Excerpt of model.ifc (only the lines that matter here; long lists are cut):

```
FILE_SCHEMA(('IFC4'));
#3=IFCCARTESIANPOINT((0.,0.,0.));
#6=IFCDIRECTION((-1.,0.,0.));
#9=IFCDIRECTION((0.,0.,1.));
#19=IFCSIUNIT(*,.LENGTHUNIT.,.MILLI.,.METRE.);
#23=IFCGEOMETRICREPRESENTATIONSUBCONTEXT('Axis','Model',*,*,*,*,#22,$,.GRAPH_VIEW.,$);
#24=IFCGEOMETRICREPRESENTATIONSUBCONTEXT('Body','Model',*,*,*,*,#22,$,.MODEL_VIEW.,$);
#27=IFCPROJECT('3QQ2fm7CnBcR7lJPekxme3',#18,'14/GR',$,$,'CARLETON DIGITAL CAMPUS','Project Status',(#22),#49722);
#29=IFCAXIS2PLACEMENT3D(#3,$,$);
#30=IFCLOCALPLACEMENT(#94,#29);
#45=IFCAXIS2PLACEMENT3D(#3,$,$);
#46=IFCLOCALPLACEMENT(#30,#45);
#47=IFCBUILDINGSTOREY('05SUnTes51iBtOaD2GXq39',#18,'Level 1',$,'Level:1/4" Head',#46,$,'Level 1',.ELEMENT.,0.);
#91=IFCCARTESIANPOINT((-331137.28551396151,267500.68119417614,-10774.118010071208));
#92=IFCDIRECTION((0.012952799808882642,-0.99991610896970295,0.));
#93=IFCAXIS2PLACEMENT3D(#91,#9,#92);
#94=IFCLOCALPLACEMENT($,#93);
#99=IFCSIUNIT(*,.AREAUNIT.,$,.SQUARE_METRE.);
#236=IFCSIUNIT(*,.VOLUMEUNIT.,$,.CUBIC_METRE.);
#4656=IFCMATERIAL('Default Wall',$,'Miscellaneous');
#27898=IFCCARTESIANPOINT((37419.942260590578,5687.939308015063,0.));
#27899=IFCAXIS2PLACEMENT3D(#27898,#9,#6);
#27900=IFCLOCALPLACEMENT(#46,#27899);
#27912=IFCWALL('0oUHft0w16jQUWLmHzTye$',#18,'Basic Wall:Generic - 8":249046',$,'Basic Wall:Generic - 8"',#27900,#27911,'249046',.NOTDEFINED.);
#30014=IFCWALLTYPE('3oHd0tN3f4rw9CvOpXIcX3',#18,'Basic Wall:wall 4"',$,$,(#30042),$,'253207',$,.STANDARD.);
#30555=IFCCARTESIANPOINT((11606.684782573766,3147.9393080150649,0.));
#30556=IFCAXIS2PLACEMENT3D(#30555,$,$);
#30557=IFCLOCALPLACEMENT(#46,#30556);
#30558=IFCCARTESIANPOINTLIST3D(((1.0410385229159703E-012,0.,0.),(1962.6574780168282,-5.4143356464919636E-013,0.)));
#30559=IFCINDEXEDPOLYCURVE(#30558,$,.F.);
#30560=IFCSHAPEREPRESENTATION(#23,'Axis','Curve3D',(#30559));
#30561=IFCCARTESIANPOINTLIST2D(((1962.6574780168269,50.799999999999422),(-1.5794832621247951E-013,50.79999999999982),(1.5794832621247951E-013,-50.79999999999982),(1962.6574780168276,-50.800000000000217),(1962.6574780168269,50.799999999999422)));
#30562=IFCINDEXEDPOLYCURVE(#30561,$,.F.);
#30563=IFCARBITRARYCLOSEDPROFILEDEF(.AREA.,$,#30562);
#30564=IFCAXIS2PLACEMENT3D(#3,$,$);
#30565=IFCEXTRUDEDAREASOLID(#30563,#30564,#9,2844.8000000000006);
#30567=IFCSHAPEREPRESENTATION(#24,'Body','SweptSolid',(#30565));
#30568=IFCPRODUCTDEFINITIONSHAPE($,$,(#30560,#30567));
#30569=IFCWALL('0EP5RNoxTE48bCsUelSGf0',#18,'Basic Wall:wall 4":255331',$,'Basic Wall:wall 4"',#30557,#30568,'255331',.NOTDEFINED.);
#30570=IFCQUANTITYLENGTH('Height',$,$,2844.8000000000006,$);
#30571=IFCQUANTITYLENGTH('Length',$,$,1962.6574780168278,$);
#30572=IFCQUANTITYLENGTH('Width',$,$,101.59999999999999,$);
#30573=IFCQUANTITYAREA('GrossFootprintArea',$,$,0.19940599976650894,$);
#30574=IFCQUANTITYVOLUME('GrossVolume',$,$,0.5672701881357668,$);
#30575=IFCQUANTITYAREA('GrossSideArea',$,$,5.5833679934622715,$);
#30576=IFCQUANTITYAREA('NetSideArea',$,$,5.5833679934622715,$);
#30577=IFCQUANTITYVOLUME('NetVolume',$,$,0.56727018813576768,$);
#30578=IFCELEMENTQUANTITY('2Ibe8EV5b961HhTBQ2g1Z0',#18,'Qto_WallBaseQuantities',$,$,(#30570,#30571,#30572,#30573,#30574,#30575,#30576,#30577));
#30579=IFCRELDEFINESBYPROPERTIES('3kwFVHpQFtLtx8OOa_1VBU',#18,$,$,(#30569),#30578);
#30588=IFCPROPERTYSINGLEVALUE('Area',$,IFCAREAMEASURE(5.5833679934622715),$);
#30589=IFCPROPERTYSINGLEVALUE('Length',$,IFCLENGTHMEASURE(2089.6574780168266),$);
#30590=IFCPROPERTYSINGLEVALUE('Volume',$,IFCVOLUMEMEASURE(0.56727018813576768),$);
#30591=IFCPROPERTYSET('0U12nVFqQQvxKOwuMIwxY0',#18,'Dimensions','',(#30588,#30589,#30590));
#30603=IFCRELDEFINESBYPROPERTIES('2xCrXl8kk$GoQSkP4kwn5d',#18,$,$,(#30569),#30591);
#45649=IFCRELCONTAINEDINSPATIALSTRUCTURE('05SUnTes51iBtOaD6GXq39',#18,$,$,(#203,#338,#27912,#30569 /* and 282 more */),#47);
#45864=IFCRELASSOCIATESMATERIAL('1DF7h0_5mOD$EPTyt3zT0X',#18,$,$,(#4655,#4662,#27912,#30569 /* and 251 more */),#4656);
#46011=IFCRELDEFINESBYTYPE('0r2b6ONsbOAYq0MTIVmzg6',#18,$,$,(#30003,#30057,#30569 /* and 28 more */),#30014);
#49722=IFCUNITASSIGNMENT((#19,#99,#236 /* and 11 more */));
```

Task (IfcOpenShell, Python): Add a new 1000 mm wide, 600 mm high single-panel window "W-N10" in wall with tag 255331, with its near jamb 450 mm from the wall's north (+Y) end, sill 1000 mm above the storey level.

```python
import numpy as np
import ifcopenshell
import ifcopenshell.api.feature
import ifcopenshell.api.geometry
import ifcopenshell.api.pset
import ifcopenshell.api.root
import ifcopenshell.api.spatial
import ifcopenshell.geom
import ifcopenshell.util.element
import ifcopenshell.util.placement
import ifcopenshell.util.representation
import ifcopenshell.util.shape
import ifcopenshell.util.unit

model = ifcopenshell.open("model.ifc")
unit_scale = ifcopenshell.util.unit.calculate_unit_scale(model)
area_scale = ifcopenshell.util.unit.calculate_unit_scale(model, "AREAUNIT")
volume_scale = ifcopenshell.util.unit.calculate_unit_scale(model, "VOLUMEUNIT")
settings = ifcopenshell.geom.settings()


def volume(element):
    """Net volume in cubic metres, openings subtracted."""
    shape = ifcopenshell.geom.create_shape(settings, element)
    return ifcopenshell.util.shape.get_volume(shape.geometry)


wall = model.by_guid("0EP5RNoxTE48bCsUelSGf0")
storey = ifcopenshell.util.element.get_container(wall, ifc_class="IfcBuildingStorey")
context = ifcopenshell.util.representation.get_context(model, "Model", "Body", "MODEL_VIEW")
before = volume(wall)

width, height, from_end, sill = 1, 0.6, 0.45, 1  # metres

# The wall runs along its own X axis, and the end named is its -X end.
wall_shape = ifcopenshell.geom.create_shape(settings, wall)
x, y, z = ifcopenshell.util.shape.get_vertices(wall_shape.geometry).T
start = x.min() + from_end
face, thickness = float(y.min()), float(y.max() - y.min())
wall_matrix = ifcopenshell.util.placement.get_local_placement(wall.ObjectPlacement)
level = ifcopenshell.util.placement.get_local_placement(storey.ObjectPlacement)[2, 3]


def in_wall(x, y):
    """Placement at x, y metres in the wall's axes, at sill height."""
    matrix = wall_matrix.copy()
    matrix[:, 3] = wall_matrix @ np.array([x / unit_scale, y / unit_scale, 0.0, 1.0])
    matrix[2, 3] = level + sill / unit_scale
    return matrix


# Opening: a box that overshoots both wall faces by 50 mm.
opening = ifcopenshell.api.root.create_entity(model, ifc_class="IfcOpeningElement", predefined_type="OPENING")
box = ifcopenshell.api.geometry.add_wall_representation(
    model, context=context, length=width, height=height, thickness=thickness + 0.1
)
ifcopenshell.api.geometry.assign_representation(model, product=opening, representation=box)
ifcopenshell.api.geometry.edit_object_placement(model, product=opening, matrix=in_wall(start, face - 0.05), is_si=False)
ifcopenshell.api.feature.add_feature(model, feature=opening, element=wall)

window = ifcopenshell.api.root.create_entity(model, ifc_class="IfcWindow", name="W-N10", predefined_type="WINDOW")
window.OverallWidth, window.OverallHeight = width / unit_scale, height / unit_scale
window.PartitioningType = "SINGLE_PANEL"
body = ifcopenshell.api.geometry.add_window_representation(
    model,
    context=context,
    overall_width=window.OverallWidth,
    overall_height=window.OverallHeight,
    partition_type="SINGLE_PANEL",
)
ifcopenshell.api.geometry.assign_representation(model, product=window, representation=body)
ifcopenshell.api.spatial.assign_container(model, products=[window], relating_structure=storey)
ifcopenshell.api.feature.add_filling(model, opening=opening, element=window)

# Centre the window in the wall's thickness.
ifcopenshell.api.geometry.edit_object_placement(model, product=window, matrix=in_wall(start, face), is_si=False)
window_shape = ifcopenshell.geom.create_shape(settings, window)
depth = ifcopenshell.util.shape.get_vertices(window_shape.geometry)[:, 1]
offset = face + thickness / 2 - (depth.min() + depth.max()) / 2
ifcopenshell.api.geometry.edit_object_placement(model, product=window, matrix=in_wall(start, offset), is_si=False)

after = volume(wall)

# Update the wall's stored quantities.
qto = model.by_id(ifcopenshell.util.element.get_pset(wall, "Qto_WallBaseQuantities", should_inherit=False)["id"])
ifcopenshell.api.pset.edit_qto(model, qto=qto, properties={
    "NetSideArea": after / thickness / area_scale,
    "NetVolume": after / volume_scale,
})
pset = model.by_id(ifcopenshell.util.element.get_pset(wall, "Dimensions", should_inherit=False)["id"])
ifcopenshell.api.pset.edit_pset(model, pset=pset, properties={
    "Area": model.create_entity("IfcAreaMeasure", after / thickness / area_scale),
    "Volume": model.create_entity("IfcVolumeMeasure", after / volume_scale),
})

print(f"wall volume {before:.3f} -> {after:.3f} m3")

model.write("model_v2.ifc")
```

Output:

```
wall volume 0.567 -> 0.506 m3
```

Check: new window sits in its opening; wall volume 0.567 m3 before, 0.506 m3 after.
